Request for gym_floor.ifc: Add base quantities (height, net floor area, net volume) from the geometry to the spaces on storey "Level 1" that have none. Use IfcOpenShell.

First a look at what the model holds.

```python
import ifcopenshell
import ifcopenshell.util.element
import ifcopenshell.util.unit

model = ifcopenshell.open("gym_floor.ifc")
print(model.schema)
for unit_type in ("LENGTHUNIT", "AREAUNIT", "VOLUMEUNIT"):
    print(unit_type, ifcopenshell.util.unit.calculate_unit_scale(model, unit_type))
storey = next(s for s in model.by_type("IfcBuildingStorey") if s.Name == "Level 1")
spaces = [e for e in ifcopenshell.util.element.get_decomposition(storey) if e.is_a("IfcSpace")]
for e in sorted(spaces, key=lambda e: e.id()):
    print(e.id(), e.is_a(), e.Name, list(ifcopenshell.util.element.get_psets(e, qtos_only=True)), sep=" | ")
```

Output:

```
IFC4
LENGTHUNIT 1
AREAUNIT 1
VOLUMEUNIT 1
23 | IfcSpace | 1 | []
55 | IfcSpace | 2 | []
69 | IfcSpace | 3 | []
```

```python
import ifcopenshell
import ifcopenshell.api.pset
import ifcopenshell.geom
import ifcopenshell.util.element
import ifcopenshell.util.shape
import ifcopenshell.util.unit

model = ifcopenshell.open("gym_floor.ifc")
unit_scale = ifcopenshell.util.unit.calculate_unit_scale(model)
area_scale = ifcopenshell.util.unit.calculate_unit_scale(model, "AREAUNIT")
volume_scale = ifcopenshell.util.unit.calculate_unit_scale(model, "VOLUMEUNIT")
settings = ifcopenshell.geom.settings()

storey = next(s for s in model.by_type("IfcBuildingStorey") if s.Name == "Level 1")
spaces = [e for e in ifcopenshell.util.element.get_decomposition(storey) if e.is_a("IfcSpace")]

for e in sorted(spaces, key=lambda e: e.id()):
    if ifcopenshell.util.element.get_psets(e, qtos_only=True, should_inherit=False):
        continue
    # Geometry comes back in metres, in the element's own axes.
    shape = ifcopenshell.geom.create_shape(settings, e)
    values = {
        "Height": ifcopenshell.util.shape.get_z(shape.geometry) / unit_scale,
        "NetFloorArea": ifcopenshell.util.shape.get_footprint_area(shape.geometry) / area_scale,
        "NetVolume": ifcopenshell.util.shape.get_volume(shape.geometry) / volume_scale,
    }
    qto = ifcopenshell.api.pset.add_qto(model, product=e, name="Qto_SpaceBaseQuantities")
    ifcopenshell.api.pset.edit_qto(model, qto=qto, properties=values)
    print(e.id(), {k: round(v, 3) for k, v in values.items()})

model.write("gym_floor_rev.ifc")
```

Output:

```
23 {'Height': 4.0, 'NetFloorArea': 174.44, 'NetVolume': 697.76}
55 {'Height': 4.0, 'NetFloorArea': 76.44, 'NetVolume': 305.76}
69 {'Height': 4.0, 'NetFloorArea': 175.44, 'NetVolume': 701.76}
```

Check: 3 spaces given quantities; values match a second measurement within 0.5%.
